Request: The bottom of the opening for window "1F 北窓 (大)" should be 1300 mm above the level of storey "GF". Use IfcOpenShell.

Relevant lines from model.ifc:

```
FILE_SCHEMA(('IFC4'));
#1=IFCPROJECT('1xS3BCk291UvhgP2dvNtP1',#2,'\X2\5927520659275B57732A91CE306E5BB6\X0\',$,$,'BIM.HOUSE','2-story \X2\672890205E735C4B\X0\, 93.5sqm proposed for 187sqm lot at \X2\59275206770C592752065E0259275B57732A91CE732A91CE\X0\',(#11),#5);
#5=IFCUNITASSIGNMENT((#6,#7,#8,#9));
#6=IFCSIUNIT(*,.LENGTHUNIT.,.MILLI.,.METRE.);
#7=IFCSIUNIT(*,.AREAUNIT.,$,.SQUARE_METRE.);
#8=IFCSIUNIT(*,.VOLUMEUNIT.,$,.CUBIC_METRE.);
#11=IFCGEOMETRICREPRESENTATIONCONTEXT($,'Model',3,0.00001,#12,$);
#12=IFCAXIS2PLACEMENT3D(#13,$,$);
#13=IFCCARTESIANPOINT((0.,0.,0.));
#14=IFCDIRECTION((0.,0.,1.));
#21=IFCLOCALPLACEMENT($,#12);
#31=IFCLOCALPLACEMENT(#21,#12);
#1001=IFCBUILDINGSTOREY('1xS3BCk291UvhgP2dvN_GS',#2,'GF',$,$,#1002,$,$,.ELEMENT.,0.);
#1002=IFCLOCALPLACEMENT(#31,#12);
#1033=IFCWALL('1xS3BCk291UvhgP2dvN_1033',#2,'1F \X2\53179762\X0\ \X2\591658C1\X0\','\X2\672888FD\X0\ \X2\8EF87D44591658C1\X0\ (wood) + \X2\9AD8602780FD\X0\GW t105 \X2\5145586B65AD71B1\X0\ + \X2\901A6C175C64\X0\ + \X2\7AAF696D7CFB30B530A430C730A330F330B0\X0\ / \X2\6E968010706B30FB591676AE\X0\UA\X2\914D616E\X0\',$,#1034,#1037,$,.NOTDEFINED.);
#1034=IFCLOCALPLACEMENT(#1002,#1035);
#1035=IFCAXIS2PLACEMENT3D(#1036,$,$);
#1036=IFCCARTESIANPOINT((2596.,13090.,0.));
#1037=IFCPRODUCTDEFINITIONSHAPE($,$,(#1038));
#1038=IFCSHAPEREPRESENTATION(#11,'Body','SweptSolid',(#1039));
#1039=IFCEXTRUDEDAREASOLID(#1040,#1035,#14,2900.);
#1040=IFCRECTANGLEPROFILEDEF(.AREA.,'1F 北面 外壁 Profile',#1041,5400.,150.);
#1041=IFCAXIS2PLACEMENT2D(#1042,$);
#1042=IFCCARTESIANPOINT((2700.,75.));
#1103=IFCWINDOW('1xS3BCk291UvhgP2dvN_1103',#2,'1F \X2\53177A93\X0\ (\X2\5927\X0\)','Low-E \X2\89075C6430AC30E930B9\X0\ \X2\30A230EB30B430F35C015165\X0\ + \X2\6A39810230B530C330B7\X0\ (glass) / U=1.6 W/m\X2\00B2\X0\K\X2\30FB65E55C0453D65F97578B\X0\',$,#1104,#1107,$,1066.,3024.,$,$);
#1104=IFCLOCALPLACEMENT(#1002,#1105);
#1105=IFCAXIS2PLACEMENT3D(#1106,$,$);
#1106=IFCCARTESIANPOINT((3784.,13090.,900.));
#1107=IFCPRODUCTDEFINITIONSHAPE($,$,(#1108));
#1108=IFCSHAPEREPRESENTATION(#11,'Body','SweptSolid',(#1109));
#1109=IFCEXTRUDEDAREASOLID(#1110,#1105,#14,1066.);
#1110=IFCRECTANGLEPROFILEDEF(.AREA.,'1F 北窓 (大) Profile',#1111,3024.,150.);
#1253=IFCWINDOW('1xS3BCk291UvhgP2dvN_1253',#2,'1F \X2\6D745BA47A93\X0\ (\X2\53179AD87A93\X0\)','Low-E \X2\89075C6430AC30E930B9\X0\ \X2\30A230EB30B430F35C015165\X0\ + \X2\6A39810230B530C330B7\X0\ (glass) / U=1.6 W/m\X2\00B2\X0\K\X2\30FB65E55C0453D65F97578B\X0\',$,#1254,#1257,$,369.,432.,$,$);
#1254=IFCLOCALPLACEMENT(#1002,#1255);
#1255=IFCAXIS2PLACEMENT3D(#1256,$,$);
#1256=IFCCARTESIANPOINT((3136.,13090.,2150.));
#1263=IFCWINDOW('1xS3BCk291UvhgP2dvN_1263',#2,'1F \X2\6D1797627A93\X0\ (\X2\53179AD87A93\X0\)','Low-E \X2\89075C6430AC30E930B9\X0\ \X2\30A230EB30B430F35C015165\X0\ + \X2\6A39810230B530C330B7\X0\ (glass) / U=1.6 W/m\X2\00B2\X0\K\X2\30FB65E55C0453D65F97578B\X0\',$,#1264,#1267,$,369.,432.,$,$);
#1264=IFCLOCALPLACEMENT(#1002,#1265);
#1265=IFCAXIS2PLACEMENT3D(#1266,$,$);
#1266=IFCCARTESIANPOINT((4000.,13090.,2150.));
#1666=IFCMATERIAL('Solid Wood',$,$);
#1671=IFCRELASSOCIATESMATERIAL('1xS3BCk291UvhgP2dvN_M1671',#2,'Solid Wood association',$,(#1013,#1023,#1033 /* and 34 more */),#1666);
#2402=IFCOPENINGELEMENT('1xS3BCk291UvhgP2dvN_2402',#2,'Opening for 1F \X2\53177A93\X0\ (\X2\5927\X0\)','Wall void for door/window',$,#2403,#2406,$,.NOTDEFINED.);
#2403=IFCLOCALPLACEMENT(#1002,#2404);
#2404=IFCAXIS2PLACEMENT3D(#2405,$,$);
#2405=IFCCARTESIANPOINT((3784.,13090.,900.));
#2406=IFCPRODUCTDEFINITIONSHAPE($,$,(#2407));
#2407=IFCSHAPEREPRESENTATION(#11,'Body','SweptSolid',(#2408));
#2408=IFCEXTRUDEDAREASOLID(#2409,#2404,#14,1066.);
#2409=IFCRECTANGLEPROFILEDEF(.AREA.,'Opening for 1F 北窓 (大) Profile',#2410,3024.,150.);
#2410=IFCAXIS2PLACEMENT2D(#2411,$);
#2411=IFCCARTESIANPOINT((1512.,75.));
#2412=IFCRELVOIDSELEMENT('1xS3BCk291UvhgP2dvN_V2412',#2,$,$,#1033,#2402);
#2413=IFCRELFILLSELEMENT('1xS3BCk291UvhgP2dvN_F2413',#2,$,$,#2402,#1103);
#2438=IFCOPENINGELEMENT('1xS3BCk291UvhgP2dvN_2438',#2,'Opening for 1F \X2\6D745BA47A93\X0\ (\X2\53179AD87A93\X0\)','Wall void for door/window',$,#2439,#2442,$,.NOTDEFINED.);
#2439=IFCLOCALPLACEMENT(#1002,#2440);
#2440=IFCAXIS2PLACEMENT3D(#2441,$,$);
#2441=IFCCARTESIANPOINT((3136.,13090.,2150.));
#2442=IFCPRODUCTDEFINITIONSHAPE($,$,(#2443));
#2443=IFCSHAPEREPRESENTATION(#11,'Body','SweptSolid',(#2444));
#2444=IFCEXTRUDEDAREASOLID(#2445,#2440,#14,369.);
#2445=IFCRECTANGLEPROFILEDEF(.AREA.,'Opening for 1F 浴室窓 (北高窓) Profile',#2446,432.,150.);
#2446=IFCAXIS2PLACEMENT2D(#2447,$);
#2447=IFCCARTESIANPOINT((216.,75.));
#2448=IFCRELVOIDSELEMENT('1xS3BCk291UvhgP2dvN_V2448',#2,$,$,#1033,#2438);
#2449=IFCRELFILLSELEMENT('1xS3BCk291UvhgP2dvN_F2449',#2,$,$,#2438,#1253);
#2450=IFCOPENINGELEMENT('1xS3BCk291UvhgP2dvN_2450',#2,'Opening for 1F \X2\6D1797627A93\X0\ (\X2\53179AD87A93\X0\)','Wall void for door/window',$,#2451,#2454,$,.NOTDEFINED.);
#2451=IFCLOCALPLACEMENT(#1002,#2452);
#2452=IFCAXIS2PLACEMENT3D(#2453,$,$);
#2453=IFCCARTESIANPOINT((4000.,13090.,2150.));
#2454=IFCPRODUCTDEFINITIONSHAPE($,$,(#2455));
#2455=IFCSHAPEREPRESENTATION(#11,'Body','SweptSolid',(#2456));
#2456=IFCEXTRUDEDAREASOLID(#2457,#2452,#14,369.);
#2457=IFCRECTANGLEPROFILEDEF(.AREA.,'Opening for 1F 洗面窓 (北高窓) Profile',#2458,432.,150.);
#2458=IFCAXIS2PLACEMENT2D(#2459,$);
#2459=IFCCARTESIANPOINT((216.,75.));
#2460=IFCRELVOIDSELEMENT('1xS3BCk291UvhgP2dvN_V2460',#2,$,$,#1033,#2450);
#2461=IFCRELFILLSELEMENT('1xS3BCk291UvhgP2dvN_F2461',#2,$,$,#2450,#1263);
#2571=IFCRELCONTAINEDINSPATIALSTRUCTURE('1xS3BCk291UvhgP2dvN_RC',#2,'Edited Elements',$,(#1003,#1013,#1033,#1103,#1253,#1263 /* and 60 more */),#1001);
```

```python
import numpy as np
import ifcopenshell
import ifcopenshell.api.geometry
import ifcopenshell.geom
import ifcopenshell.util.element
import ifcopenshell.util.placement
import ifcopenshell.util.shape
import ifcopenshell.util.unit

model = ifcopenshell.open("model.ifc")
unit_scale = ifcopenshell.util.unit.calculate_unit_scale(model)

window = model.by_guid("1xS3BCk291UvhgP2dvN_1103")
opening = window.FillsVoids[0].RelatingOpeningElement
storey = ifcopenshell.util.element.get_container(window, ifc_class="IfcBuildingStorey")
level = ifcopenshell.util.placement.get_local_placement(storey.ObjectPlacement)[2, 3]

# The opening's origin need not be at the sill, so measure its lowest point.
shape = ifcopenshell.geom.create_shape(ifcopenshell.geom.settings(), opening)
bottom = ifcopenshell.util.shape.get_shape_bottom_elevation(shape, shape.geometry) / unit_scale
dz = level + 1.3 / unit_scale - bottom

shift = np.array([0.0, 0.0, dz])
# The window is not placed relative to its opening, so move both.
for product in (opening, window):
    matrix = ifcopenshell.util.placement.get_local_placement(product.ObjectPlacement)
    matrix[:3, 3] += shift
    ifcopenshell.api.geometry.edit_object_placement(model, product=product, matrix=matrix, is_si=False)

print(f"moved by {dz * unit_scale:+.3f} m")

model.write("model_rev.ifc")
```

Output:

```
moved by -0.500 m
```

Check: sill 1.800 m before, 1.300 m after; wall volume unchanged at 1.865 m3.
